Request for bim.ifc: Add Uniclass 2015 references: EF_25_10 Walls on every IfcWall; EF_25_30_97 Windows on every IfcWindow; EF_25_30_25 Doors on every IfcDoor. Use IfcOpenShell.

First a look at what the model holds.

```python
import ifcopenshell

model = ifcopenshell.open("bim.ifc")
print(model.schema)
print("classifications:", [c.Name for c in model.by_type("IfcClassification")])
for ifc_class in ("IfcDoor", "IfcRoof", "IfcStair", "IfcWall", "IfcWindow"):
    print(ifc_class, len(model.by_type(ifc_class)))
```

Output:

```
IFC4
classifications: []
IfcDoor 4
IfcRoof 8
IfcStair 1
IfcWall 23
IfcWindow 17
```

```python
import ifcopenshell
import ifcopenshell.api.classification

model = ifcopenshell.open("bim.ifc")

system = ifcopenshell.api.classification.add_classification(model, classification="Uniclass 2015")

codes = {
    "IfcWall": ("EF_25_10", "Walls"),
    "IfcWindow": ("EF_25_30_97", "Windows"),
    "IfcDoor": ("EF_25_30_25", "Doors"),
}
for ifc_class, (code, name) in codes.items():
    products = model.by_type(ifc_class)
    ifcopenshell.api.classification.add_reference(
        model, products=products, classification=system, identification=code, name=name
    )
    print(code, len(products))

model.write("bim_rev.ifc")
```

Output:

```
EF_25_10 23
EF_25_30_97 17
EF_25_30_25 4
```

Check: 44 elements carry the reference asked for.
